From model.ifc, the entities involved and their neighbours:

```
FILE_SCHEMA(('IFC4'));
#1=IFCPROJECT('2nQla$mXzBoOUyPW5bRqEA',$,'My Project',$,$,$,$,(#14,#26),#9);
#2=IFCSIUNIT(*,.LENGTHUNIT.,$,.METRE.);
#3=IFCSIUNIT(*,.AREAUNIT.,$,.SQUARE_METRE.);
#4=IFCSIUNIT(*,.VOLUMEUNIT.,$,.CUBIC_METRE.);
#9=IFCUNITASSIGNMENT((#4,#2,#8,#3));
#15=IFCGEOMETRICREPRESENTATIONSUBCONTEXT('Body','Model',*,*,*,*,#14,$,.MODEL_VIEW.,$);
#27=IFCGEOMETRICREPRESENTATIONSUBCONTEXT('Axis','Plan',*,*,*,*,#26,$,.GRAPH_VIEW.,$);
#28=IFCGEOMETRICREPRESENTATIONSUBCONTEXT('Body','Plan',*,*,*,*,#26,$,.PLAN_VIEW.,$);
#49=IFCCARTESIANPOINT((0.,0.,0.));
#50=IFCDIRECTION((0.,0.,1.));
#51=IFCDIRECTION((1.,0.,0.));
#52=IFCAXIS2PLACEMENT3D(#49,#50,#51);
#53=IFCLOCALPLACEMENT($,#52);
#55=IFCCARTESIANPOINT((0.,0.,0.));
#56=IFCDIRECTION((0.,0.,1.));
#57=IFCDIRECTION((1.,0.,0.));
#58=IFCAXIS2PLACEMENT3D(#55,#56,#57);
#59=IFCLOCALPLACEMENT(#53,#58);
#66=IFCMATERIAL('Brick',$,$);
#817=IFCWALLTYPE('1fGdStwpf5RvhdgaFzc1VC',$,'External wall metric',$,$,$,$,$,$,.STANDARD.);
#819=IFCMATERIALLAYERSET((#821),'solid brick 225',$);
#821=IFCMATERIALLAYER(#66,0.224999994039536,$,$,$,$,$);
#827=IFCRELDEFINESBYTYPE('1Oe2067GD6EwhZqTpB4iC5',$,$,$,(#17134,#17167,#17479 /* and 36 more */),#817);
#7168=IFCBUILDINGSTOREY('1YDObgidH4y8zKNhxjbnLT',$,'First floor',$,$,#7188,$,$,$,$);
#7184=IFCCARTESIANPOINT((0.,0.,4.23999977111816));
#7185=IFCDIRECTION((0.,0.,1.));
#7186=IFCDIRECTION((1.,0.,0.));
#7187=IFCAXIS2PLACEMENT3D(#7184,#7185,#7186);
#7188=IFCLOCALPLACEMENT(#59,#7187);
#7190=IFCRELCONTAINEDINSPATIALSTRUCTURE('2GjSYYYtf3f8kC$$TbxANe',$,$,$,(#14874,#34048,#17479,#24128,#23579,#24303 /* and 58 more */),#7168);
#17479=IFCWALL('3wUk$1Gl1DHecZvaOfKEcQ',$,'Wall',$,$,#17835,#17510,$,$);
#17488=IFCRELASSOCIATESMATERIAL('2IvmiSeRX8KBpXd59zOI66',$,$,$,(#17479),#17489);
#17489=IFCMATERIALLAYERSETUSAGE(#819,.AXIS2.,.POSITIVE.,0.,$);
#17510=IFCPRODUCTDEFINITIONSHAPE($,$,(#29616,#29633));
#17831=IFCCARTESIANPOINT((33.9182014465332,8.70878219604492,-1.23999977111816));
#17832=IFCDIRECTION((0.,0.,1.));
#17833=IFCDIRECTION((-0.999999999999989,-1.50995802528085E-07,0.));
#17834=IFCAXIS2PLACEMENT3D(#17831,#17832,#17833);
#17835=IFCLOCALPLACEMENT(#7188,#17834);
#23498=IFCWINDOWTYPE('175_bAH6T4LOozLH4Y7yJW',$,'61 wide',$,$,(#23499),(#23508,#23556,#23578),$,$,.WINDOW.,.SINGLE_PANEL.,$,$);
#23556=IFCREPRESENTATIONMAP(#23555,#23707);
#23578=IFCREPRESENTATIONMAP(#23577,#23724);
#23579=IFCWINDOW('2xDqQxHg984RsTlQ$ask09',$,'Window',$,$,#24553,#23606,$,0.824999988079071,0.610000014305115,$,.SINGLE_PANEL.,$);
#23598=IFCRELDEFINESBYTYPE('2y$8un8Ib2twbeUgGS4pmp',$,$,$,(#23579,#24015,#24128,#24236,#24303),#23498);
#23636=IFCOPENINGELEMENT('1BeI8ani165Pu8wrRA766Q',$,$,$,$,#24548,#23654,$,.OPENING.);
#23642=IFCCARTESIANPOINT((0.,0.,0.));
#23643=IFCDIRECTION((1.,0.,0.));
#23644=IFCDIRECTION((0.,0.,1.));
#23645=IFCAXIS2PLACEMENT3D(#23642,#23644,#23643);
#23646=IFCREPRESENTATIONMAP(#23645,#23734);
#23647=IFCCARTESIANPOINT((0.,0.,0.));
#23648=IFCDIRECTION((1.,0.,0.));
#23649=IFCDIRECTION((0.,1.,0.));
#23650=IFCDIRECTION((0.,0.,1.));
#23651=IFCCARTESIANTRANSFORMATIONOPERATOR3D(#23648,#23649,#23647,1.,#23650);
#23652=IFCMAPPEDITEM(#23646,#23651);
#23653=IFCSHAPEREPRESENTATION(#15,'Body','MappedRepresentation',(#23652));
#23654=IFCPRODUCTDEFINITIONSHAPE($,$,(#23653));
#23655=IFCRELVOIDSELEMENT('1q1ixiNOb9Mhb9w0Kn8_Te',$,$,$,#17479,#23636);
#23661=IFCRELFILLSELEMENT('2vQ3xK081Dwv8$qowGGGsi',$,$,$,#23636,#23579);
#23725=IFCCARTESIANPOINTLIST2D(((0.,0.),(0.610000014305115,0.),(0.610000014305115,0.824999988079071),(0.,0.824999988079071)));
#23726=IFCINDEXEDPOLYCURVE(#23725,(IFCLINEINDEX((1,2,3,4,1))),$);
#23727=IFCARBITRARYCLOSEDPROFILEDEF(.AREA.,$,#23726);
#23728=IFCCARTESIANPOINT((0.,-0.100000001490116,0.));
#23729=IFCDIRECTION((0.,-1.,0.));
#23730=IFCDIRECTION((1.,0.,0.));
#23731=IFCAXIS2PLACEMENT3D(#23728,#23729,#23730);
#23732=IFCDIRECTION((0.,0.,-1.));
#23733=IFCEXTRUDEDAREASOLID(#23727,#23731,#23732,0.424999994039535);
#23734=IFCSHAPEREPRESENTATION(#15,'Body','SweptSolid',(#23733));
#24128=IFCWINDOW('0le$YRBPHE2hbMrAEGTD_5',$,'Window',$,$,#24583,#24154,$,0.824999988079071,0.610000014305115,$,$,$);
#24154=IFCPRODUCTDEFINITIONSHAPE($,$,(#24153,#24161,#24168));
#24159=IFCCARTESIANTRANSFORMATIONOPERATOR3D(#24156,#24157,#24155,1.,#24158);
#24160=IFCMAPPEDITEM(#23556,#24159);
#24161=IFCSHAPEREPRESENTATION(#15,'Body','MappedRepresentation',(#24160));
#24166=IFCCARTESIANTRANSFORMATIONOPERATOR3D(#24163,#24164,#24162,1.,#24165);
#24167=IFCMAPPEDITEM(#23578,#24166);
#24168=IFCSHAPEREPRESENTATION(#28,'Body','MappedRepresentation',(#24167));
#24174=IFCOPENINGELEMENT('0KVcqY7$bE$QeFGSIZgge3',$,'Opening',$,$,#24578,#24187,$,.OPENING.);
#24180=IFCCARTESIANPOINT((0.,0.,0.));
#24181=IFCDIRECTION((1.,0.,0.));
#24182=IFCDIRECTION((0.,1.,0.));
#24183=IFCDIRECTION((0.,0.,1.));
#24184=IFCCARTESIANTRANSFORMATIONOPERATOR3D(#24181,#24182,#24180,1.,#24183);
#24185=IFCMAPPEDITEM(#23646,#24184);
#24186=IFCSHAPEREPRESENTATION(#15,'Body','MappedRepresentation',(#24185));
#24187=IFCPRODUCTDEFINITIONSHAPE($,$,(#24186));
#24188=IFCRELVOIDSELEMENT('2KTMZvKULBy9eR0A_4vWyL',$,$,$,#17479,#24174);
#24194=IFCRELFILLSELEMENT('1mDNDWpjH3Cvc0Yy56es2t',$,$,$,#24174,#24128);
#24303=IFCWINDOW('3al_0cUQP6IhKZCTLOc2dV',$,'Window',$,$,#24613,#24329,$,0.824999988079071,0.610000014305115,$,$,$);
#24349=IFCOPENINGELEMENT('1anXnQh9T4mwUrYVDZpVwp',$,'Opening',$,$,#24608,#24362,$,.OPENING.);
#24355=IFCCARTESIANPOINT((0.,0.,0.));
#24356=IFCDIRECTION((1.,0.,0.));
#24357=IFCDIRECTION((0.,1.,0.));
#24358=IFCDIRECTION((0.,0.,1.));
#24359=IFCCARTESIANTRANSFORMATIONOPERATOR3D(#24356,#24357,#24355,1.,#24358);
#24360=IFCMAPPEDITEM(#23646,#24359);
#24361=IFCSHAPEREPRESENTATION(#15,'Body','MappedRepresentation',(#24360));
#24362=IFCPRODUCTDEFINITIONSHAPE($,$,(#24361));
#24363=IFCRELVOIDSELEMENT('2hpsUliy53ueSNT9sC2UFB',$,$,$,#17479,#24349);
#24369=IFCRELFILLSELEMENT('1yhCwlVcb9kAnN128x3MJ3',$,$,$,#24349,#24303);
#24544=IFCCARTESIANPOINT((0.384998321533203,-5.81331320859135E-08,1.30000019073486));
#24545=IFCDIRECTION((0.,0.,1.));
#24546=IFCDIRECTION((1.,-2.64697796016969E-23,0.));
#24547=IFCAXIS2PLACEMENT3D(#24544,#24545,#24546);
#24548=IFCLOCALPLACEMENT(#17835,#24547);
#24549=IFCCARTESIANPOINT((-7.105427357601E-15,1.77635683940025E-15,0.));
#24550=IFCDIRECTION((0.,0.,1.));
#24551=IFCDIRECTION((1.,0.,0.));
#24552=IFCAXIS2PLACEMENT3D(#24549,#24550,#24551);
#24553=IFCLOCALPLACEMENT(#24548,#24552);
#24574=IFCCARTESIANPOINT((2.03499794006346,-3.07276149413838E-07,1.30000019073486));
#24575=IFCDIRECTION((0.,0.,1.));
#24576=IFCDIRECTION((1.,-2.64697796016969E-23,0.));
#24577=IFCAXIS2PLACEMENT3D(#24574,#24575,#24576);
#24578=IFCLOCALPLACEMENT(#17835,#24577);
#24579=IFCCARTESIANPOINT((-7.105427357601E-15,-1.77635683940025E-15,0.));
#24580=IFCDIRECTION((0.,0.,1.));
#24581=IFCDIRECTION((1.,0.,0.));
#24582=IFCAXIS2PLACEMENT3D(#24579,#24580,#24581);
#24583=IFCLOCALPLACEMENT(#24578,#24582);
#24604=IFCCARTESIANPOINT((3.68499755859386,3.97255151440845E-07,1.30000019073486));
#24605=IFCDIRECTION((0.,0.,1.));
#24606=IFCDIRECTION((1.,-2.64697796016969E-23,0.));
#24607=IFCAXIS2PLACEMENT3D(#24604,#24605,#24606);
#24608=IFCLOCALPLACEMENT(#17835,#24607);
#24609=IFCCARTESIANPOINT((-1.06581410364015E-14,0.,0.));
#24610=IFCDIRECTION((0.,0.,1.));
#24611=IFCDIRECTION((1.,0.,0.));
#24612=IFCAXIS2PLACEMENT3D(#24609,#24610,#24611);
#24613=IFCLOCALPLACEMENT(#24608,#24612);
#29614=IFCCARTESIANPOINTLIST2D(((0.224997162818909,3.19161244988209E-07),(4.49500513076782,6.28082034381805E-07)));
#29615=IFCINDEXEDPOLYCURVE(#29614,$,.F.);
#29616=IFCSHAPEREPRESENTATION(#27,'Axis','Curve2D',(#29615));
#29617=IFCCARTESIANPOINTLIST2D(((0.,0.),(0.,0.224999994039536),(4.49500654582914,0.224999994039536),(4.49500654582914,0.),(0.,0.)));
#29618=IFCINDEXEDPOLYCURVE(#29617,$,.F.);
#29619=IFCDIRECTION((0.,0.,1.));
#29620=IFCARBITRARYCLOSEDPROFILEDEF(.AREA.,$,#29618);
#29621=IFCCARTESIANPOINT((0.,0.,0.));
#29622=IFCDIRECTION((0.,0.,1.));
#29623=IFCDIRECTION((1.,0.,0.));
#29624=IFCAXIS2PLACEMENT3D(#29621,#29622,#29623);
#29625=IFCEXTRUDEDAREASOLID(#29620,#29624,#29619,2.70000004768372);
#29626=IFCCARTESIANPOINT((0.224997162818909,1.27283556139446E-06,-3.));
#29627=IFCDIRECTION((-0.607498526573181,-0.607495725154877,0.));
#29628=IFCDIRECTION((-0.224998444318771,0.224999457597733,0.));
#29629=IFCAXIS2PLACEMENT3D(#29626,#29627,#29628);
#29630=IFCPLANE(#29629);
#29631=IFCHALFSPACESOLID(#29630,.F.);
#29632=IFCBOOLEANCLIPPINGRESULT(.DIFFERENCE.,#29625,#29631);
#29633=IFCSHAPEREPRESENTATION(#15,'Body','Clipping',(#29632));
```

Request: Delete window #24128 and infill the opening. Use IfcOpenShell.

```python
import ifcopenshell
import ifcopenshell.api.feature
import ifcopenshell.api.root
import ifcopenshell.geom
import ifcopenshell.util.shape

model = ifcopenshell.open("model.ifc")
settings = ifcopenshell.geom.settings()


def volume(element):
    """Net volume in cubic metres, openings subtracted."""
    shape = ifcopenshell.geom.create_shape(settings, element)
    return ifcopenshell.util.shape.get_volume(shape.geometry)


window = model.by_id(24128)
opening = window.FillsVoids[0].RelatingOpeningElement
wall = opening.VoidsElements[0].RelatingBuildingElement
before = volume(wall)

ifcopenshell.api.root.remove_product(model, product=window)
ifcopenshell.api.feature.remove_feature(model, feature=opening)

after = volume(wall)

print(f"wall volume {before:.3f} -> {after:.3f} m3")

model.write("model_v2.ifc")
```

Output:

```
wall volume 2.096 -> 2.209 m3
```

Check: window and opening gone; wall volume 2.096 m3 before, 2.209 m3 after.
